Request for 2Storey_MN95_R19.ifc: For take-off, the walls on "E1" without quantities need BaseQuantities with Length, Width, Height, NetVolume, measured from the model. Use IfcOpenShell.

First a look at what the model holds.

```python
import ifcopenshell
import ifcopenshell.util.element
import ifcopenshell.util.unit

model = ifcopenshell.open("2Storey_MN95_R19.ifc")
print(model.schema)
for unit_type in ("LENGTHUNIT", "AREAUNIT", "VOLUMEUNIT"):
    print(unit_type, ifcopenshell.util.unit.calculate_unit_scale(model, unit_type))
storey = next(s for s in model.by_type("IfcBuildingStorey") if s.Name == "E1")
walls = [e for e in ifcopenshell.util.element.get_decomposition(storey) if e.is_a("IfcWall")]
for e in sorted(walls, key=lambda e: e.id()):
    print(e.id(), e.is_a(), e.Name, list(ifcopenshell.util.element.get_psets(e, qtos_only=True)), sep=" | ")
```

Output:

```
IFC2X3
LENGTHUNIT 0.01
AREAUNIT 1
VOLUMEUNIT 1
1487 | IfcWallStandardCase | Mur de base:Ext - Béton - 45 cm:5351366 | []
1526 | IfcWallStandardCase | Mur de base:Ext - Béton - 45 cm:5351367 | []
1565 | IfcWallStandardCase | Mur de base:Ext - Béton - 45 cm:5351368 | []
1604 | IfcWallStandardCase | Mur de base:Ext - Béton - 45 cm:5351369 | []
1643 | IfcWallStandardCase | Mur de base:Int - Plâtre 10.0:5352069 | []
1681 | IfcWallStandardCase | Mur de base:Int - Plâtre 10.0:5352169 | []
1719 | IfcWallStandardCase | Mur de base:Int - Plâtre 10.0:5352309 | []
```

```python
import ifcopenshell
import ifcopenshell.api.pset
import ifcopenshell.geom
import ifcopenshell.util.element
import ifcopenshell.util.shape
import ifcopenshell.util.unit

model = ifcopenshell.open("2Storey_MN95_R19.ifc")
unit_scale = ifcopenshell.util.unit.calculate_unit_scale(model)
volume_scale = ifcopenshell.util.unit.calculate_unit_scale(model, "VOLUMEUNIT")
settings = ifcopenshell.geom.settings()

storey = next(s for s in model.by_type("IfcBuildingStorey") if s.Name == "E1")
walls = [e for e in ifcopenshell.util.element.get_decomposition(storey) if e.is_a("IfcWall")]

for e in sorted(walls, key=lambda e: e.id()):
    if ifcopenshell.util.element.get_psets(e, qtos_only=True, should_inherit=False):
        continue
    # Geometry comes back in metres, in the element's own axes.
    shape = ifcopenshell.geom.create_shape(settings, e)
    values = {
        "Length": ifcopenshell.util.shape.get_x(shape.geometry) / unit_scale,
        "Width": ifcopenshell.util.shape.get_y(shape.geometry) / unit_scale,
        "Height": ifcopenshell.util.shape.get_z(shape.geometry) / unit_scale,
        "NetVolume": ifcopenshell.util.shape.get_volume(shape.geometry) / volume_scale,
    }
    qto = ifcopenshell.api.pset.add_qto(model, product=e, name="BaseQuantities")
    ifcopenshell.api.pset.edit_qto(model, qto=qto, properties=values)
    print(e.id(), {k: round(v, 3) for k, v in values.items()})

model.write("2Storey_MN95_R19_updated.ifc")
```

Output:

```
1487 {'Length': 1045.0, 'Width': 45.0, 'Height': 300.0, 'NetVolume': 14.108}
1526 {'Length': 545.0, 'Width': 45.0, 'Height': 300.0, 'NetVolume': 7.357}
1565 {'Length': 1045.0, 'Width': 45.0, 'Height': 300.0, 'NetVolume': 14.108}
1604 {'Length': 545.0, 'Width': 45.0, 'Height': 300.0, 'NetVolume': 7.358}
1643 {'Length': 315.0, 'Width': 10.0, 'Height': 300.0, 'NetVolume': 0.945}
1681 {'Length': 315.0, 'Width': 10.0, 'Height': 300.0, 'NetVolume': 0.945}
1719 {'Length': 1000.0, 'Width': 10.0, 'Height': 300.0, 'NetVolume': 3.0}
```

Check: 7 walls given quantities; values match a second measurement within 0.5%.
